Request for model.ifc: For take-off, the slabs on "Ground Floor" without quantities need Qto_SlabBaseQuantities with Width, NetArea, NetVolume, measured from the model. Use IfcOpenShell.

First a look at what the model holds.

```python
import ifcopenshell
import ifcopenshell.util.element
import ifcopenshell.util.unit

model = ifcopenshell.open("model.ifc")
print(model.schema)
for unit_type in ("LENGTHUNIT", "AREAUNIT", "VOLUMEUNIT"):
    print(unit_type, ifcopenshell.util.unit.calculate_unit_scale(model, unit_type))
storey = next(s for s in model.by_type("IfcBuildingStorey") if s.Name == "Ground Floor")
slabs = [e for e in ifcopenshell.util.element.get_decomposition(storey) if e.is_a("IfcSlab")]
for e in sorted(slabs, key=lambda e: e.id()):
    print(e.id(), e.is_a(), e.Name, list(ifcopenshell.util.element.get_psets(e, qtos_only=True)), sep=" | ")
```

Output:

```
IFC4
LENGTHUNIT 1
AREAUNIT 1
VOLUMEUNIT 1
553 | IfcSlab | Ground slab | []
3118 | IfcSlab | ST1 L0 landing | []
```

```python
import ifcopenshell
import ifcopenshell.api.pset
import ifcopenshell.geom
import ifcopenshell.util.element
import ifcopenshell.util.shape
import ifcopenshell.util.unit

model = ifcopenshell.open("model.ifc")
unit_scale = ifcopenshell.util.unit.calculate_unit_scale(model)
area_scale = ifcopenshell.util.unit.calculate_unit_scale(model, "AREAUNIT")
volume_scale = ifcopenshell.util.unit.calculate_unit_scale(model, "VOLUMEUNIT")
settings = ifcopenshell.geom.settings()

storey = next(s for s in model.by_type("IfcBuildingStorey") if s.Name == "Ground Floor")
slabs = [e for e in ifcopenshell.util.element.get_decomposition(storey) if e.is_a("IfcSlab")]

for e in sorted(slabs, key=lambda e: e.id()):
    if ifcopenshell.util.element.get_psets(e, qtos_only=True, should_inherit=False):
        continue
    # Geometry comes back in metres, in the element's own axes.
    shape = ifcopenshell.geom.create_shape(settings, e)
    values = {
        "Width": ifcopenshell.util.shape.get_z(shape.geometry) / unit_scale,
        "NetArea": ifcopenshell.util.shape.get_footprint_area(shape.geometry) / area_scale,
        "NetVolume": ifcopenshell.util.shape.get_volume(shape.geometry) / volume_scale,
    }
    qto = ifcopenshell.api.pset.add_qto(model, product=e, name="Qto_SlabBaseQuantities")
    ifcopenshell.api.pset.edit_qto(model, qto=qto, properties=values)
    print(e.id(), {k: round(v, 3) for k, v in values.items()})

model.write("model_v2.ifc")
```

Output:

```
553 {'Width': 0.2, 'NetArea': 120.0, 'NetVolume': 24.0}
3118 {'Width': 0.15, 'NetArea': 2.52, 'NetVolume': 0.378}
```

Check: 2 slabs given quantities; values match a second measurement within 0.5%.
